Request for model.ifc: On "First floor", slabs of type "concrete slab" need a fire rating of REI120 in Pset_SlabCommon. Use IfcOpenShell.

First a look at what the model holds.

```python
import ifcopenshell
import ifcopenshell.util.element

model = ifcopenshell.open("model.ifc")
print(model.schema)
storey = next(s for s in model.by_type("IfcBuildingStorey") if s.Name == "First floor")
slabs = [e for e in ifcopenshell.util.element.get_decomposition(storey) if e.is_a("IfcSlab")]
seen = {}
for e in slabs:
    element_type = ifcopenshell.util.element.get_type(e)
    key = (element_type.Name if element_type != e and element_type else None, ifcopenshell.util.element.get_pset(e, "Pset_SlabCommon", "FireRating"))
    seen[key] = seen.get(key, 0) + 1
for (name, value), count in sorted(seen.items(), key=str):
    print(count, "x", name, "|", value)
```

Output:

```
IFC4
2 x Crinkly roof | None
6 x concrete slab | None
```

```python
import ifcopenshell
import ifcopenshell.api.pset
import ifcopenshell.util.element

model = ifcopenshell.open("model.ifc")

storey = next(s for s in model.by_type("IfcBuildingStorey") if s.Name == "First floor")
slabs = [e for e in ifcopenshell.util.element.get_decomposition(storey) if e.is_a("IfcSlab")]

count = 0
for e in slabs:
    element_type = ifcopenshell.util.element.get_type(e)
    if element_type in (None, e) or element_type.Name != "concrete slab":
        continue
    # add_pset returns the element's existing set when there is one.
    pset = ifcopenshell.api.pset.add_pset(model, product=e, name="Pset_SlabCommon")
    ifcopenshell.api.pset.edit_pset(model, pset=pset, properties={"FireRating": "REI120"})
    count += 1

print(count, "slabs updated")

model.write("model_updated.ifc")
```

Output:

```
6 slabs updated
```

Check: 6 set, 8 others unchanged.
